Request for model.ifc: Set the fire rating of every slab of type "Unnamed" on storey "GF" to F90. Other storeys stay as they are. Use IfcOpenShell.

First a look at what the model holds.

```python
import ifcopenshell
import ifcopenshell.util.element

model = ifcopenshell.open("model.ifc")
print(model.schema)
storey = next(s for s in model.by_type("IfcBuildingStorey") if s.Name == "GF")
slabs = [e for e in ifcopenshell.util.element.get_decomposition(storey) if e.is_a("IfcSlab")]
seen = {}
for e in slabs:
    element_type = ifcopenshell.util.element.get_type(e)
    key = (element_type.Name if element_type != e and element_type else None, ifcopenshell.util.element.get_pset(e, "Pset_SlabCommon", "FireRating"))
    seen[key] = seen.get(key, 0) + 1
for (name, value), count in sorted(seen.items(), key=str):
    print(count, "x", name, "|", value)
```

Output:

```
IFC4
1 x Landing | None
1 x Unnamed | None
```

```python
import ifcopenshell
import ifcopenshell.api.pset
import ifcopenshell.util.element

model = ifcopenshell.open("model.ifc")

storey = next(s for s in model.by_type("IfcBuildingStorey") if s.Name == "GF")
slabs = [e for e in ifcopenshell.util.element.get_decomposition(storey) if e.is_a("IfcSlab")]

count = 0
for e in slabs:
    element_type = ifcopenshell.util.element.get_type(e)
    if element_type in (None, e) or element_type.Name != "Unnamed":
        continue
    # add_pset returns the element's existing set when there is one.
    pset = ifcopenshell.api.pset.add_pset(model, product=e, name="Pset_SlabCommon")
    ifcopenshell.api.pset.edit_pset(model, pset=pset, properties={"FireRating": "F90"})
    count += 1

print(count, "slabs updated")

model.write("model_rev.ifc")
```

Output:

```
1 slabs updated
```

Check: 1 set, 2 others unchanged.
